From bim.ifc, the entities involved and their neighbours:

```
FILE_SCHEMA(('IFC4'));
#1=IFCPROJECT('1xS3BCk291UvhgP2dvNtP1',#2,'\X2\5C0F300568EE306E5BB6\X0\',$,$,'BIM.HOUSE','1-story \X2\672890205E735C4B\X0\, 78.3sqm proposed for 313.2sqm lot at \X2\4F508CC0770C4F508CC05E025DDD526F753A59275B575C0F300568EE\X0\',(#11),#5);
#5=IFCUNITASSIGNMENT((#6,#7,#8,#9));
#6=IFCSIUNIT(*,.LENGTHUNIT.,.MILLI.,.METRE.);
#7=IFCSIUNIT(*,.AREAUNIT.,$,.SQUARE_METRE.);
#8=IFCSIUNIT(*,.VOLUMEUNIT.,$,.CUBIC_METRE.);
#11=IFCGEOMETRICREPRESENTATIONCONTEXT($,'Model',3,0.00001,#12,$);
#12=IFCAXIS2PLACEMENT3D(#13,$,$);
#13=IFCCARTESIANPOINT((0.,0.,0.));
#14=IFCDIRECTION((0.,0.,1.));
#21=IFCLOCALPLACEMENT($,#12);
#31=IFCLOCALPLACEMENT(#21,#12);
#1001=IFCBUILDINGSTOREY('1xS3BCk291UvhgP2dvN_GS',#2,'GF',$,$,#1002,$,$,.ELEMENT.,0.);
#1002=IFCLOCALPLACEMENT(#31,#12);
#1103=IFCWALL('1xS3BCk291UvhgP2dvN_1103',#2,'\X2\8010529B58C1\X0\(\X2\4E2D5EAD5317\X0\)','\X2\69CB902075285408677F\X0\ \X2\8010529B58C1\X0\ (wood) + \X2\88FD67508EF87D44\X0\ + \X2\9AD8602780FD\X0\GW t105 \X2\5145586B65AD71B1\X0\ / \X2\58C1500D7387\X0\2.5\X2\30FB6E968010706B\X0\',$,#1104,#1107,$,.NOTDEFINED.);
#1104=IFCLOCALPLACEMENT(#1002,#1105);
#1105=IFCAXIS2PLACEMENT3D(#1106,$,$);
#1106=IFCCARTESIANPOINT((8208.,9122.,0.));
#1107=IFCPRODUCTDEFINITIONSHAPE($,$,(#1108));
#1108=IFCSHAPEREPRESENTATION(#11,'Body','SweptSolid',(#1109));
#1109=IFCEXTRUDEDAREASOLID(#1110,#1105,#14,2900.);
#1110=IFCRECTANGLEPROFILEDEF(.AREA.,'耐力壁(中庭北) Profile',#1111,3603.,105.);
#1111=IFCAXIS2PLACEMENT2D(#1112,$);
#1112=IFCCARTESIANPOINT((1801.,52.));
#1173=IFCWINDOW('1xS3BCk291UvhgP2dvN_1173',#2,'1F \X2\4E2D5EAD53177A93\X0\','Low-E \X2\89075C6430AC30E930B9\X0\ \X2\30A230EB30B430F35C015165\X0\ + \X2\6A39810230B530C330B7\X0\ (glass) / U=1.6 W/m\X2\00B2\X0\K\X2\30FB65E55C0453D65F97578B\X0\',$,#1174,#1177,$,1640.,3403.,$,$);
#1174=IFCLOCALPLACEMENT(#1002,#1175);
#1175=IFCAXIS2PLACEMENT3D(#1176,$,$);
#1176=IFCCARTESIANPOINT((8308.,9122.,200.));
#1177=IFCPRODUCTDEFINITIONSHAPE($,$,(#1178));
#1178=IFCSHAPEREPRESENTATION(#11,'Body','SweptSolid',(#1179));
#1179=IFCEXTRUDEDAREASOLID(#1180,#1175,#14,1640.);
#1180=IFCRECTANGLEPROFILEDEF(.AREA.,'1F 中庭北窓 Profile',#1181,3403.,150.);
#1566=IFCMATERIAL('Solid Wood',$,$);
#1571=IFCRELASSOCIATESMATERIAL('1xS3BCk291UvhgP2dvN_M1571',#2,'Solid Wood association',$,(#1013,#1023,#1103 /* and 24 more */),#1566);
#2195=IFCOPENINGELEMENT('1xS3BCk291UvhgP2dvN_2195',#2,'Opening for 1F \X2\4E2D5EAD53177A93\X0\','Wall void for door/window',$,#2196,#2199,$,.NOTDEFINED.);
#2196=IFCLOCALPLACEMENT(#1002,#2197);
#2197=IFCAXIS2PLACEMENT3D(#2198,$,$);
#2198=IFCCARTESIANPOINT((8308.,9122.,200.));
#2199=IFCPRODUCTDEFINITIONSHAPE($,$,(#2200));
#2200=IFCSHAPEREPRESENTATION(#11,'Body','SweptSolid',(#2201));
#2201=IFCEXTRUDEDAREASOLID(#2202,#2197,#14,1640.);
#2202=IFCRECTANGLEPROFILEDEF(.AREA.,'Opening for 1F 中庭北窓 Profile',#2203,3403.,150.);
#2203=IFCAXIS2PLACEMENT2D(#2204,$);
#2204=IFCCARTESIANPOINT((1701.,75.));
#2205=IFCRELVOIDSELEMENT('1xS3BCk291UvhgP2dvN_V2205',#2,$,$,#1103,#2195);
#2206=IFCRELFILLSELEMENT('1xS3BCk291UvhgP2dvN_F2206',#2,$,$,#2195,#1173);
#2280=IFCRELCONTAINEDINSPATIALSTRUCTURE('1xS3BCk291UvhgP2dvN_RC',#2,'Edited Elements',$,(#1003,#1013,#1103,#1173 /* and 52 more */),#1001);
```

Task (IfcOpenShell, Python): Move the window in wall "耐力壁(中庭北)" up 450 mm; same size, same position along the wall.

```python
import numpy as np
import ifcopenshell
import ifcopenshell.api.geometry
import ifcopenshell.util.placement
import ifcopenshell.util.unit

model = ifcopenshell.open("bim.ifc")
unit_scale = ifcopenshell.util.unit.calculate_unit_scale(model)

window = model.by_guid("1xS3BCk291UvhgP2dvN_1173")
opening = window.FillsVoids[0].RelatingOpeningElement
dz = 0.45 / unit_scale

shift = np.array([0.0, 0.0, dz])
# The window is not placed relative to its opening, so move both.
for product in (opening, window):
    matrix = ifcopenshell.util.placement.get_local_placement(product.ObjectPlacement)
    matrix[:3, 3] += shift
    ifcopenshell.api.geometry.edit_object_placement(model, product=product, matrix=matrix, is_si=False)

print(f"moved by {dz * unit_scale:+.3f} m")

model.write("bim_updated.ifc")
```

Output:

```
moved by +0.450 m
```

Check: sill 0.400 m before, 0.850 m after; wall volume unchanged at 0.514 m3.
